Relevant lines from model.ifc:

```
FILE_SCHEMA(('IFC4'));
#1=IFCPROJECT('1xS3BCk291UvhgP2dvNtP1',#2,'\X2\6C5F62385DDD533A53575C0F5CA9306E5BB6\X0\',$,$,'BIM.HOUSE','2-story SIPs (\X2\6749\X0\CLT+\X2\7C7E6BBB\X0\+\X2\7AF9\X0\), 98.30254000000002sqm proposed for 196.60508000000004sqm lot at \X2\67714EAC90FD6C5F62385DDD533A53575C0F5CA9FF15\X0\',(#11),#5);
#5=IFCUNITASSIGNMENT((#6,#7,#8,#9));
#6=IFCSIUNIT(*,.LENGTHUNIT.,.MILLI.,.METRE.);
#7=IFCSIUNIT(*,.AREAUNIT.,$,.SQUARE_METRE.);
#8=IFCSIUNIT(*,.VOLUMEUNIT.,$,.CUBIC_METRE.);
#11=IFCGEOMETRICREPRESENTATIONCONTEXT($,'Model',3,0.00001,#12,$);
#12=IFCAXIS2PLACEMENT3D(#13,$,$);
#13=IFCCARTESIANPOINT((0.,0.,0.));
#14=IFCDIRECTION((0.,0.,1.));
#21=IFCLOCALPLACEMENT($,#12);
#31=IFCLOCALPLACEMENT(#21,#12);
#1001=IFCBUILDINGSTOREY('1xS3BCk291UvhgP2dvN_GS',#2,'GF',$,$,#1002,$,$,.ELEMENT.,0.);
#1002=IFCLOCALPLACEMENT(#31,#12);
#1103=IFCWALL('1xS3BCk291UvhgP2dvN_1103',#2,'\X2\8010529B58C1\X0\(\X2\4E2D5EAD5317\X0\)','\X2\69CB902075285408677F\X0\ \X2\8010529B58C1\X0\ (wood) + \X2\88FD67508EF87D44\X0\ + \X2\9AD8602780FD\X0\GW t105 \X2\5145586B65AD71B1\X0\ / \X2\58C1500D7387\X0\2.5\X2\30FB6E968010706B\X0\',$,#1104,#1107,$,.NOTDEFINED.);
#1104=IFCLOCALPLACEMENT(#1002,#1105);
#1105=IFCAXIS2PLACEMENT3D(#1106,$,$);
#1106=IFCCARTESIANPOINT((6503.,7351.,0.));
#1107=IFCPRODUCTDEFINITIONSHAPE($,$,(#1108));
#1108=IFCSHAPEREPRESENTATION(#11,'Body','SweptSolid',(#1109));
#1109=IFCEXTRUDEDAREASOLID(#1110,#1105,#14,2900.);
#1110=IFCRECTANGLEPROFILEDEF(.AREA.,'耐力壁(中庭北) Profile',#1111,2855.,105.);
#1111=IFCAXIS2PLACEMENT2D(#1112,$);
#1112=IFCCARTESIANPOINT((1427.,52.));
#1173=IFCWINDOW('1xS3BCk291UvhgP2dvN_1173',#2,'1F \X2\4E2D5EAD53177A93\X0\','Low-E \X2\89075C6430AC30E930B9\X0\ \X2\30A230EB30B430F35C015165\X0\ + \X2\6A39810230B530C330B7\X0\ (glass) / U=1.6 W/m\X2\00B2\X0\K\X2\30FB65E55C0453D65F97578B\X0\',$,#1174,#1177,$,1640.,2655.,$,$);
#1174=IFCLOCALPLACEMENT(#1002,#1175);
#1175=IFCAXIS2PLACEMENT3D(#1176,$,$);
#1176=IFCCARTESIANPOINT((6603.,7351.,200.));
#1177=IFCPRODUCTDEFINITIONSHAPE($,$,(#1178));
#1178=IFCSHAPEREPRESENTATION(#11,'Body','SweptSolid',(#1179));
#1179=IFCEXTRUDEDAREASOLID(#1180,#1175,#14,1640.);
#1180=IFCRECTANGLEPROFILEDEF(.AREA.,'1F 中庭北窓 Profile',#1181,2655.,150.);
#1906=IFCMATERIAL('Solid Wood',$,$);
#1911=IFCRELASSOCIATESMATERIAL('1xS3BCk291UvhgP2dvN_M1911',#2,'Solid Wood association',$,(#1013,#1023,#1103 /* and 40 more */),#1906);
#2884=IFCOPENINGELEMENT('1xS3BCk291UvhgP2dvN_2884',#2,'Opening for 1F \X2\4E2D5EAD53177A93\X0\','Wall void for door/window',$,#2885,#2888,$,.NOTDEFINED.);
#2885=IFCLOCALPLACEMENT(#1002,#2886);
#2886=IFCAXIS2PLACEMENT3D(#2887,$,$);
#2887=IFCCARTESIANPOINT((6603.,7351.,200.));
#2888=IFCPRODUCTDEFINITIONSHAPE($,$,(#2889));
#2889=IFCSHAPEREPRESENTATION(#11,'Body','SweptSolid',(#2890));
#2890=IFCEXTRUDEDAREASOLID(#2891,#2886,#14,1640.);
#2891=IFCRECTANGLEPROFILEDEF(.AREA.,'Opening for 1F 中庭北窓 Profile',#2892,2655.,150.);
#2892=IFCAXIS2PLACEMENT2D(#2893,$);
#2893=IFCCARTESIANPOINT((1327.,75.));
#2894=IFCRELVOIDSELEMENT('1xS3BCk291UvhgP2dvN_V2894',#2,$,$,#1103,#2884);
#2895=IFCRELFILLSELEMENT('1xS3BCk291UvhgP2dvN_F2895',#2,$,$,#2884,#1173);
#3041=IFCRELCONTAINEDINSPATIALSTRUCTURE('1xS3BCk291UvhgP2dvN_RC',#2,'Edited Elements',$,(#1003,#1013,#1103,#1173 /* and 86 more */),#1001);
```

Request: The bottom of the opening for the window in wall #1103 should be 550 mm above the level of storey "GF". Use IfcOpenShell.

```python
import numpy as np
import ifcopenshell
import ifcopenshell.api.geometry
import ifcopenshell.geom
import ifcopenshell.util.element
import ifcopenshell.util.placement
import ifcopenshell.util.shape
import ifcopenshell.util.unit

model = ifcopenshell.open("model.ifc")
unit_scale = ifcopenshell.util.unit.calculate_unit_scale(model)

window = model.by_guid("1xS3BCk291UvhgP2dvN_1173")
opening = window.FillsVoids[0].RelatingOpeningElement
storey = ifcopenshell.util.element.get_container(window, ifc_class="IfcBuildingStorey")
level = ifcopenshell.util.placement.get_local_placement(storey.ObjectPlacement)[2, 3]

# The opening's origin need not be at the sill, so measure its lowest point.
shape = ifcopenshell.geom.create_shape(ifcopenshell.geom.settings(), opening)
bottom = ifcopenshell.util.shape.get_shape_bottom_elevation(shape, shape.geometry) / unit_scale
dz = level + 0.55 / unit_scale - bottom

shift = np.array([0.0, 0.0, dz])
# The window is not placed relative to its opening, so move both.
for product in (opening, window):
    matrix = ifcopenshell.util.placement.get_local_placement(product.ObjectPlacement)
    matrix[:3, 3] += shift
    ifcopenshell.api.geometry.edit_object_placement(model, product=product, matrix=matrix, is_si=False)

print(f"moved by {dz * unit_scale:+.3f} m")

model.write("model_edited.ifc")
```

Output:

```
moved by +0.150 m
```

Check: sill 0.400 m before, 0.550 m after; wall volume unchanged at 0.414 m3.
